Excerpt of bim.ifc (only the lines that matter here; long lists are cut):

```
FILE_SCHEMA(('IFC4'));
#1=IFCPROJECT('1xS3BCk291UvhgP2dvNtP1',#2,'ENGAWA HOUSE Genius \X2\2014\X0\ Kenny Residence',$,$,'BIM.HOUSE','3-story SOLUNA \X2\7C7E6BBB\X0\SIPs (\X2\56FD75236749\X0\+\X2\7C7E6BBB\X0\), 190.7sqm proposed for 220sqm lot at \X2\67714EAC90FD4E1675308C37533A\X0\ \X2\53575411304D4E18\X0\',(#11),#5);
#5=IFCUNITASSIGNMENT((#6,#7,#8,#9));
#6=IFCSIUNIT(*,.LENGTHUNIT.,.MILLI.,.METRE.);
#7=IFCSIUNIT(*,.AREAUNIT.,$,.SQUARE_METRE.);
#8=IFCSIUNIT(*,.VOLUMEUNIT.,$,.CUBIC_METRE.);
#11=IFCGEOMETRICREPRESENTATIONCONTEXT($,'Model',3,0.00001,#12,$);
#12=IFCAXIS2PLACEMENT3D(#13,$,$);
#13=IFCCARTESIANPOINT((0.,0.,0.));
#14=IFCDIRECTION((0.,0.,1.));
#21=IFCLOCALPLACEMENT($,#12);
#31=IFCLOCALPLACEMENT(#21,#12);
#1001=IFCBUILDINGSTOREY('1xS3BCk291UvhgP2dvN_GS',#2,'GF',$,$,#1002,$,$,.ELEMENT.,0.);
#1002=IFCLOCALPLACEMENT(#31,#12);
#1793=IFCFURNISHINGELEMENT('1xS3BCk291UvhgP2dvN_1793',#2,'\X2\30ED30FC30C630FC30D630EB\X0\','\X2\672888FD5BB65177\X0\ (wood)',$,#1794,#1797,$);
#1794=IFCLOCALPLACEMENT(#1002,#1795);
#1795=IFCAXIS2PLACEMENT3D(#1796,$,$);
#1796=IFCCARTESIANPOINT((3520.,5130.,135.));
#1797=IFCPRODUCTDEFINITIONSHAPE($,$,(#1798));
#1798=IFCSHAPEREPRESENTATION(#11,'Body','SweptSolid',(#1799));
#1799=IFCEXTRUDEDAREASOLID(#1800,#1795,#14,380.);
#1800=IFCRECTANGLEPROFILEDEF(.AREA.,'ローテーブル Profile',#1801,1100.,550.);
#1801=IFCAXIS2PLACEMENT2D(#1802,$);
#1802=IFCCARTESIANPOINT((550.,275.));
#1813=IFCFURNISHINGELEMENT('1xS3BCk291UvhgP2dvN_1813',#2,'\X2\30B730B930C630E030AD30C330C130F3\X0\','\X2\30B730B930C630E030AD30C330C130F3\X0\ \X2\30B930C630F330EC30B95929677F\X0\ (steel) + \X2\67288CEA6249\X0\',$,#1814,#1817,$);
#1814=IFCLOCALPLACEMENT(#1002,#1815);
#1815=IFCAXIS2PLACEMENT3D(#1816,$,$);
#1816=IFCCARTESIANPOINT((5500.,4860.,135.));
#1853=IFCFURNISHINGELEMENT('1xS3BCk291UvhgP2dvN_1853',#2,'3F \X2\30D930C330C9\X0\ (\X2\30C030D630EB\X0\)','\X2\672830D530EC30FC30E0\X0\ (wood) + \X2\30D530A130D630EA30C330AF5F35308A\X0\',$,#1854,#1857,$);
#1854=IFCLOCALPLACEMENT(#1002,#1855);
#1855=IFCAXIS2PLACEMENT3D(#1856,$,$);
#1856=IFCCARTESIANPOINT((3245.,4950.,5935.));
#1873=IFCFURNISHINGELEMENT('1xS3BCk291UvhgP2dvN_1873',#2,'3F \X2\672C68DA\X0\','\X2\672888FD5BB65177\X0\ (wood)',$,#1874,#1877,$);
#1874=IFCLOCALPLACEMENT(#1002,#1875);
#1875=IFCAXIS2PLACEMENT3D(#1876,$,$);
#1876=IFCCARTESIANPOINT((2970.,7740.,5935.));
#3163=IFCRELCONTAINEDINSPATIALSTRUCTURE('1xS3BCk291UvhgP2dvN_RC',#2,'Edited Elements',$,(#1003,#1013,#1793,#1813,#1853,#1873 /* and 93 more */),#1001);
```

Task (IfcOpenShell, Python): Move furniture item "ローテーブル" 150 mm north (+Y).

```python
import ifcopenshell
import ifcopenshell.api.geometry
import ifcopenshell.util.placement

model = ifcopenshell.open("bim.ifc")

item = model.by_id(1793)
matrix = ifcopenshell.util.placement.get_local_placement(item.ObjectPlacement)
matrix[1, 3] += 150.0
ifcopenshell.api.geometry.edit_object_placement(model, product=item, matrix=matrix, is_si=False)

print(ifcopenshell.util.placement.get_local_placement(item.ObjectPlacement).round(3) + 0.0)

model.write("bim-out.ifc")
```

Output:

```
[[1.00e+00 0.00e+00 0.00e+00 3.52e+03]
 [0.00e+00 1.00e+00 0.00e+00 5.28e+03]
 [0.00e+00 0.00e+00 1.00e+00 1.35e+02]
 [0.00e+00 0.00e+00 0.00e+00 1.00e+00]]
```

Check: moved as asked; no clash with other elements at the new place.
